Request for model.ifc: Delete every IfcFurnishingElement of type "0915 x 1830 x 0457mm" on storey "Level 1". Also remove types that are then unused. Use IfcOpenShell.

First a look at what the model holds.

```python
import ifcopenshell
import ifcopenshell.util.element

model = ifcopenshell.open("model.ifc")
print(model.schema)
storey = next(s for s in model.by_type("IfcBuildingStorey") if s.Name == "Level 1")
furniture = [e for e in ifcopenshell.util.element.get_decomposition(storey) if e.is_a("IfcFurnishingElement")]
seen = {}
for e in furniture:
    element_type = ifcopenshell.util.element.get_type(e)
    name = element_type.Name if element_type not in (None, e) else None
    seen[name] = seen.get(name, 0) + 1
for name, count in sorted(seen.items(), key=str):
    print(count, "x", name)
```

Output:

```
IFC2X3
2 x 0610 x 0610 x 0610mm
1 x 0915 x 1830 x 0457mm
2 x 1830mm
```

```python
import ifcopenshell
import ifcopenshell.api.root
import ifcopenshell.util.element

model = ifcopenshell.open("model.ifc")

storey = next(s for s in model.by_type("IfcBuildingStorey") if s.Name == "Level 1")
furniture = [e for e in ifcopenshell.util.element.get_decomposition(storey) if e.is_a("IfcFurnishingElement")]
targets = [e for e in furniture if (t := ifcopenshell.util.element.get_type(e)) not in (None, e) and t.Name == "0915 x 1830 x 0457mm"]
types = {ifcopenshell.util.element.get_type(e) for e in targets} - {None, *targets}

for e in targets:
    ifcopenshell.api.root.remove_product(model, product=e)
print(len(targets), "removed")

unused = [t for t in types if not ifcopenshell.util.element.get_types(t)]
for t in unused:
    ifcopenshell.api.root.remove_product(model, product=t)
print(len(unused), "unused types removed")

model.write("model_updated.ifc")
```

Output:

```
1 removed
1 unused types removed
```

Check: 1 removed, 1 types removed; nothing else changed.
